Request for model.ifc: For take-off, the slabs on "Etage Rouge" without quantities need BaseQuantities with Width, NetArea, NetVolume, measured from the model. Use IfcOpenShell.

First a look at what the model holds.

```python
import ifcopenshell
import ifcopenshell.util.element
import ifcopenshell.util.unit

model = ifcopenshell.open("model.ifc")
print(model.schema)
for unit_type in ("LENGTHUNIT", "AREAUNIT", "VOLUMEUNIT"):
    print(unit_type, ifcopenshell.util.unit.calculate_unit_scale(model, unit_type))
storey = next(s for s in model.by_type("IfcBuildingStorey") if s.Name == "Etage Rouge")
slabs = [e for e in ifcopenshell.util.element.get_decomposition(storey) if e.is_a("IfcSlab")]
for e in sorted(slabs, key=lambda e: e.id()):
    print(e.id(), e.is_a(), e.Name, list(ifcopenshell.util.element.get_psets(e, qtos_only=True)), sep=" | ")
```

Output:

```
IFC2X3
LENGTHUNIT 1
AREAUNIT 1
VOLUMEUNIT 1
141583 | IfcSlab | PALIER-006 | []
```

```python
import ifcopenshell
import ifcopenshell.api.pset
import ifcopenshell.geom
import ifcopenshell.util.element
import ifcopenshell.util.shape
import ifcopenshell.util.unit

model = ifcopenshell.open("model.ifc")
unit_scale = ifcopenshell.util.unit.calculate_unit_scale(model)
area_scale = ifcopenshell.util.unit.calculate_unit_scale(model, "AREAUNIT")
volume_scale = ifcopenshell.util.unit.calculate_unit_scale(model, "VOLUMEUNIT")
settings = ifcopenshell.geom.settings()

storey = next(s for s in model.by_type("IfcBuildingStorey") if s.Name == "Etage Rouge")
slabs = [e for e in ifcopenshell.util.element.get_decomposition(storey) if e.is_a("IfcSlab")]

for e in sorted(slabs, key=lambda e: e.id()):
    if ifcopenshell.util.element.get_psets(e, qtos_only=True, should_inherit=False):
        continue
    # Geometry comes back in metres, in the element's own axes.
    shape = ifcopenshell.geom.create_shape(settings, e)
    values = {
        "Width": ifcopenshell.util.shape.get_z(shape.geometry) / unit_scale,
        "NetArea": ifcopenshell.util.shape.get_footprint_area(shape.geometry) / area_scale,
        "NetVolume": ifcopenshell.util.shape.get_volume(shape.geometry) / volume_scale,
    }
    qto = ifcopenshell.api.pset.add_qto(model, product=e, name="BaseQuantities")
    ifcopenshell.api.pset.edit_qto(model, qto=qto, properties=values)
    print(e.id(), {k: round(v, 3) for k, v in values.items()})

model.write("model_rev.ifc")
```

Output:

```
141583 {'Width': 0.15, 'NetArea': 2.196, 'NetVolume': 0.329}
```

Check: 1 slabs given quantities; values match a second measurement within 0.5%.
